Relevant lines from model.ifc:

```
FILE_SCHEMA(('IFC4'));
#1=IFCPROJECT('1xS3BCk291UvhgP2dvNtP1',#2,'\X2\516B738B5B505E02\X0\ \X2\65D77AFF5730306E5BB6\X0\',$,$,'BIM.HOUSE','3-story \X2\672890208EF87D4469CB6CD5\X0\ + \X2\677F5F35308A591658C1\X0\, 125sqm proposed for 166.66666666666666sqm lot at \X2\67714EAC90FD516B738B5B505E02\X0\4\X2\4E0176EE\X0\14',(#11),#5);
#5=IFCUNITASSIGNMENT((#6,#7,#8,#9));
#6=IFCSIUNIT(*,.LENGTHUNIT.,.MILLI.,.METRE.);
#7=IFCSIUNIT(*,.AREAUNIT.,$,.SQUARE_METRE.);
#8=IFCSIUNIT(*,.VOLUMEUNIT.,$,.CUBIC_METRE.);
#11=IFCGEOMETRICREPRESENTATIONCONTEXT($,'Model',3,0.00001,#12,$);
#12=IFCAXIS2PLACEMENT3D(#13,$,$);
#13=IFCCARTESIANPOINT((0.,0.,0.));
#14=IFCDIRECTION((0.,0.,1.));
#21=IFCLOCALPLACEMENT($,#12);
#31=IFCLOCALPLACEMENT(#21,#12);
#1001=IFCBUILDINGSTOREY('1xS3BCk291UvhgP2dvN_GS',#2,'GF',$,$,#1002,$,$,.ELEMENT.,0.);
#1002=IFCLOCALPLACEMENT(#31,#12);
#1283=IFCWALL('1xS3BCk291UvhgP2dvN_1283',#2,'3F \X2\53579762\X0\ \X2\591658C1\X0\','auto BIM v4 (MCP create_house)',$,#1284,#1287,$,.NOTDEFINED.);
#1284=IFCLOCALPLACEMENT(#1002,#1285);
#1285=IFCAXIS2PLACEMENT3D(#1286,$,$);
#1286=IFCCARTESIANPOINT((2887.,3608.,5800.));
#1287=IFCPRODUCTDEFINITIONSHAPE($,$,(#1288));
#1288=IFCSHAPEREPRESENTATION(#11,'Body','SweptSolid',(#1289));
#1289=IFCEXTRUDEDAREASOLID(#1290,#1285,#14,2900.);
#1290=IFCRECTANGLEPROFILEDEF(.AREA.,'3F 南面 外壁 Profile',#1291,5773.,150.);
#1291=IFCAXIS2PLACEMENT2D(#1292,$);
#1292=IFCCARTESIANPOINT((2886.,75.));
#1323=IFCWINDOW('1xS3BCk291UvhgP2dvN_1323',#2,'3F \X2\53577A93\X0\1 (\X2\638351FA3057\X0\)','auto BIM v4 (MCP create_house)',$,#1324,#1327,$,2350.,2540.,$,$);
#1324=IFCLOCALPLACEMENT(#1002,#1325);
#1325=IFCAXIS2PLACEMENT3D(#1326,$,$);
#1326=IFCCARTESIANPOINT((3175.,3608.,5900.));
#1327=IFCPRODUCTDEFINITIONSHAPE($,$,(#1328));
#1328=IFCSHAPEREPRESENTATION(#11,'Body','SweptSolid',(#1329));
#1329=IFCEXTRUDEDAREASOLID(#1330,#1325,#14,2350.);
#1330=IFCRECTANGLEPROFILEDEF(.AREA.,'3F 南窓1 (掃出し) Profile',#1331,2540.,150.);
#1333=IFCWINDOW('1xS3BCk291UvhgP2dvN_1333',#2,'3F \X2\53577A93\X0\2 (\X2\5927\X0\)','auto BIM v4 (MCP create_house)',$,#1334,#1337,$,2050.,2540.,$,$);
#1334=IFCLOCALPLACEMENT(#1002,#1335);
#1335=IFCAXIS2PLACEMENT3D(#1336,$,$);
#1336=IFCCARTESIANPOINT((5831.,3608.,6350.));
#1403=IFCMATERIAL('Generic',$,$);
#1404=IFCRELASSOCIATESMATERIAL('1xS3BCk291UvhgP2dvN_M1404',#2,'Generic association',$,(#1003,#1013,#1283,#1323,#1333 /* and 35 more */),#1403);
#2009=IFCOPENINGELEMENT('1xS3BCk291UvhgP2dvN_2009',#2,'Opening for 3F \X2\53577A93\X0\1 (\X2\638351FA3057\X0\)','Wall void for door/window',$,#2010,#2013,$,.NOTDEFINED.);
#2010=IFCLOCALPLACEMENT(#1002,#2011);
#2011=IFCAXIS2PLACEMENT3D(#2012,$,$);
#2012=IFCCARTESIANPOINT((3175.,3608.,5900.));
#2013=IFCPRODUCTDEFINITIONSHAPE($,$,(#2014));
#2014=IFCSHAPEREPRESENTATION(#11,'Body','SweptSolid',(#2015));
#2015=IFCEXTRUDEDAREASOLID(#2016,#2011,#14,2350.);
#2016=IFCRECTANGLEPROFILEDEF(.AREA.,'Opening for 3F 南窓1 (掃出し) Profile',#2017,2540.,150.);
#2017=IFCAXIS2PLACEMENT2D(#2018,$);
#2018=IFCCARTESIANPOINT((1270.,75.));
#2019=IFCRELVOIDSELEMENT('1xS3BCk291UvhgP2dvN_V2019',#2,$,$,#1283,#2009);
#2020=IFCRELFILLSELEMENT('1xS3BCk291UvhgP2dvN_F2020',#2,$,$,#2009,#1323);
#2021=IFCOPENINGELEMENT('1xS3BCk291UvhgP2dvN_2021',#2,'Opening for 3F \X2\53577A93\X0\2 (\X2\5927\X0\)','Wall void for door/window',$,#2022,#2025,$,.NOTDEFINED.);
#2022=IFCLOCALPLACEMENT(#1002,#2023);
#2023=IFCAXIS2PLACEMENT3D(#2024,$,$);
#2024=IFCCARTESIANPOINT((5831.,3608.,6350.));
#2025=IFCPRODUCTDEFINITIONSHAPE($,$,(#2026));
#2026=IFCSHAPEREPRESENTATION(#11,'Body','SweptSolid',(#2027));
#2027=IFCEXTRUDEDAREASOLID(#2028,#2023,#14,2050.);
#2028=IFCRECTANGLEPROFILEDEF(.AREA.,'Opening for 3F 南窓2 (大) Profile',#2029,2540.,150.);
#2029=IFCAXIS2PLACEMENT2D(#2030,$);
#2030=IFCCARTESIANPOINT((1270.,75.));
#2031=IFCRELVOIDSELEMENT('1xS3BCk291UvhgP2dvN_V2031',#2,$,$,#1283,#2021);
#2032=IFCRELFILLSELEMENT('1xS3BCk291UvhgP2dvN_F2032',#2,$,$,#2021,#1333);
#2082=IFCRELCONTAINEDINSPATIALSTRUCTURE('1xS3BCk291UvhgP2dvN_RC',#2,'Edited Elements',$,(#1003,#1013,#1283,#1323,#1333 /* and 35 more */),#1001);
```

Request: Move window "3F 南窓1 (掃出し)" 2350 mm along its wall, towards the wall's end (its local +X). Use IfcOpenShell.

```python
import ifcopenshell
import ifcopenshell.api.geometry
import ifcopenshell.util.placement

model = ifcopenshell.open("model.ifc")

window = model.by_guid("1xS3BCk291UvhgP2dvN_1323")
opening = window.FillsVoids[0].RelatingOpeningElement
wall = opening.VoidsElements[0].RelatingBuildingElement

wall_matrix = ifcopenshell.util.placement.get_local_placement(wall.ObjectPlacement)
shift = wall_matrix[:3, 0] * 2350.0
before = ifcopenshell.util.placement.get_local_placement(window.ObjectPlacement)[:3, 3].copy()

# The window is not placed relative to its opening, so move both.
for product in (opening, window):
    matrix = ifcopenshell.util.placement.get_local_placement(product.ObjectPlacement)
    matrix[:3, 3] += shift
    ifcopenshell.api.geometry.edit_object_placement(model, product=product, matrix=matrix, is_si=False)

after = ifcopenshell.util.placement.get_local_placement(window.ObjectPlacement)[:3, 3]
print("window moved by", (after - before).round(3) + 0.0)

model.write("model_rev.ifc")
```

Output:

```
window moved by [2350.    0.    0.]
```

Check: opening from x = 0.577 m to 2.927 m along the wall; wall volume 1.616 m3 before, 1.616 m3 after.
